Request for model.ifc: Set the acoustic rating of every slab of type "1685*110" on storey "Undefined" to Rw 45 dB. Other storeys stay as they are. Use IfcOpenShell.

First a look at what the model holds.

```python
import ifcopenshell
import ifcopenshell.util.element

model = ifcopenshell.open("model.ifc")
print(model.schema)
storey = next(s for s in model.by_type("IfcBuildingStorey") if s.Name == "Undefined")
slabs = [e for e in ifcopenshell.util.element.get_decomposition(storey) if e.is_a("IfcSlab")]
seen = {}
for e in slabs:
    element_type = ifcopenshell.util.element.get_type(e)
    key = (element_type.Name if element_type != e and element_type else None, ifcopenshell.util.element.get_pset(e, "Pset_SlabCommon", "AcousticRating"))
    seen[key] = seen.get(key, 0) + 1
for (name, value), count in sorted(seen.items(), key=str):
    print(count, "x", name, "|", value)
```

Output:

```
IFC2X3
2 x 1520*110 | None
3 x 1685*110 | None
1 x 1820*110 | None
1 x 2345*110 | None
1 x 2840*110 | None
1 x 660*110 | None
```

```python
import ifcopenshell
import ifcopenshell.api.pset
import ifcopenshell.util.element

model = ifcopenshell.open("model.ifc")

storey = next(s for s in model.by_type("IfcBuildingStorey") if s.Name == "Undefined")
slabs = [e for e in ifcopenshell.util.element.get_decomposition(storey) if e.is_a("IfcSlab")]

count = 0
for e in slabs:
    element_type = ifcopenshell.util.element.get_type(e)
    if element_type in (None, e) or element_type.Name != "1685*110":
        continue
    # add_pset returns the element's existing set when there is one.
    pset = ifcopenshell.api.pset.add_pset(model, product=e, name="Pset_SlabCommon")
    ifcopenshell.api.pset.edit_pset(model, pset=pset, properties={"AcousticRating": "Rw 45 dB"})
    count += 1

print(count, "slabs updated")

model.write("model_v2.ifc")
```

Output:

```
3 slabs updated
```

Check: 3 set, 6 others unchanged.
